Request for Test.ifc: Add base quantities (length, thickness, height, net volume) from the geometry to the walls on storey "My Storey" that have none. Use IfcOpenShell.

First a look at what the model holds.

```python
import ifcopenshell
import ifcopenshell.util.element
import ifcopenshell.util.unit

model = ifcopenshell.open("Test.ifc")
print(model.schema)
for unit_type in ("LENGTHUNIT", "AREAUNIT", "VOLUMEUNIT"):
    print(unit_type, ifcopenshell.util.unit.calculate_unit_scale(model, unit_type))
storey = next(s for s in model.by_type("IfcBuildingStorey") if s.Name == "My Storey")
walls = [e for e in ifcopenshell.util.element.get_decomposition(storey) if e.is_a("IfcWall")]
for e in sorted(walls, key=lambda e: e.id()):
    print(e.id(), e.is_a(), e.Name, list(ifcopenshell.util.element.get_psets(e, qtos_only=True)), sep=" | ")
```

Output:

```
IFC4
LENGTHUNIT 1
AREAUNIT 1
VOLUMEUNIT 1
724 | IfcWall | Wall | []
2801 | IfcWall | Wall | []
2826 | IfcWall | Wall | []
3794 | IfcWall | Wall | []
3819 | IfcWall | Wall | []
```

```python
import ifcopenshell
import ifcopenshell.api.pset
import ifcopenshell.geom
import ifcopenshell.util.element
import ifcopenshell.util.shape
import ifcopenshell.util.unit

model = ifcopenshell.open("Test.ifc")
unit_scale = ifcopenshell.util.unit.calculate_unit_scale(model)
volume_scale = ifcopenshell.util.unit.calculate_unit_scale(model, "VOLUMEUNIT")
settings = ifcopenshell.geom.settings()

storey = next(s for s in model.by_type("IfcBuildingStorey") if s.Name == "My Storey")
walls = [e for e in ifcopenshell.util.element.get_decomposition(storey) if e.is_a("IfcWall")]

for e in sorted(walls, key=lambda e: e.id()):
    if ifcopenshell.util.element.get_psets(e, qtos_only=True, should_inherit=False):
        continue
    # Geometry comes back in metres, in the element's own axes.
    shape = ifcopenshell.geom.create_shape(settings, e)
    values = {
        "Length": ifcopenshell.util.shape.get_x(shape.geometry) / unit_scale,
        "Width": ifcopenshell.util.shape.get_y(shape.geometry) / unit_scale,
        "Height": ifcopenshell.util.shape.get_z(shape.geometry) / unit_scale,
        "NetVolume": ifcopenshell.util.shape.get_volume(shape.geometry) / volume_scale,
    }
    qto = ifcopenshell.api.pset.add_qto(model, product=e, name="Qto_WallBaseQuantities")
    ifcopenshell.api.pset.edit_qto(model, qto=qto, properties=values)
    print(e.id(), {k: round(v, 3) for k, v in values.items()})

model.write("Test_edited.ifc")
```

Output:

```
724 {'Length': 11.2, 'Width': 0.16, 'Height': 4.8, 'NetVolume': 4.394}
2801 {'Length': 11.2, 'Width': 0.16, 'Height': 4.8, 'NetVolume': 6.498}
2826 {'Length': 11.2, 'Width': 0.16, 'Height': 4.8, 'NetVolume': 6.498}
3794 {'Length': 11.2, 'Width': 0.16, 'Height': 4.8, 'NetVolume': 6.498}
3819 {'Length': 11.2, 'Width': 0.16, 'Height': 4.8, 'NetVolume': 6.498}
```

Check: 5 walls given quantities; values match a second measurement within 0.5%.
